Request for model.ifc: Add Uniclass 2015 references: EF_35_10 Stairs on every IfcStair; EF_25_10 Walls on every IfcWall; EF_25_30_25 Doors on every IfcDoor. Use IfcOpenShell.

First a look at what the model holds.

```python
import ifcopenshell

model = ifcopenshell.open("model.ifc")
print(model.schema)
print("classifications:", [c.Name for c in model.by_type("IfcClassification")])
for ifc_class in ("IfcDoor", "IfcRoof", "IfcStair", "IfcWall", "IfcWindow"):
    print(ifc_class, len(model.by_type(ifc_class)))
```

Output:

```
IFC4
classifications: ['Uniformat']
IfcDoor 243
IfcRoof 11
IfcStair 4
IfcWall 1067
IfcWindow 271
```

```python
import ifcopenshell
import ifcopenshell.api.classification

model = ifcopenshell.open("model.ifc")

system = ifcopenshell.api.classification.add_classification(model, classification="Uniclass 2015")

codes = {
    "IfcStair": ("EF_35_10", "Stairs"),
    "IfcWall": ("EF_25_10", "Walls"),
    "IfcDoor": ("EF_25_30_25", "Doors"),
}
for ifc_class, (code, name) in codes.items():
    products = model.by_type(ifc_class)
    ifcopenshell.api.classification.add_reference(
        model, products=products, classification=system, identification=code, name=name
    )
    print(code, len(products))

model.write("model_edited.ifc")
```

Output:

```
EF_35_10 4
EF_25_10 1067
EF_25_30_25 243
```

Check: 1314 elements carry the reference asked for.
